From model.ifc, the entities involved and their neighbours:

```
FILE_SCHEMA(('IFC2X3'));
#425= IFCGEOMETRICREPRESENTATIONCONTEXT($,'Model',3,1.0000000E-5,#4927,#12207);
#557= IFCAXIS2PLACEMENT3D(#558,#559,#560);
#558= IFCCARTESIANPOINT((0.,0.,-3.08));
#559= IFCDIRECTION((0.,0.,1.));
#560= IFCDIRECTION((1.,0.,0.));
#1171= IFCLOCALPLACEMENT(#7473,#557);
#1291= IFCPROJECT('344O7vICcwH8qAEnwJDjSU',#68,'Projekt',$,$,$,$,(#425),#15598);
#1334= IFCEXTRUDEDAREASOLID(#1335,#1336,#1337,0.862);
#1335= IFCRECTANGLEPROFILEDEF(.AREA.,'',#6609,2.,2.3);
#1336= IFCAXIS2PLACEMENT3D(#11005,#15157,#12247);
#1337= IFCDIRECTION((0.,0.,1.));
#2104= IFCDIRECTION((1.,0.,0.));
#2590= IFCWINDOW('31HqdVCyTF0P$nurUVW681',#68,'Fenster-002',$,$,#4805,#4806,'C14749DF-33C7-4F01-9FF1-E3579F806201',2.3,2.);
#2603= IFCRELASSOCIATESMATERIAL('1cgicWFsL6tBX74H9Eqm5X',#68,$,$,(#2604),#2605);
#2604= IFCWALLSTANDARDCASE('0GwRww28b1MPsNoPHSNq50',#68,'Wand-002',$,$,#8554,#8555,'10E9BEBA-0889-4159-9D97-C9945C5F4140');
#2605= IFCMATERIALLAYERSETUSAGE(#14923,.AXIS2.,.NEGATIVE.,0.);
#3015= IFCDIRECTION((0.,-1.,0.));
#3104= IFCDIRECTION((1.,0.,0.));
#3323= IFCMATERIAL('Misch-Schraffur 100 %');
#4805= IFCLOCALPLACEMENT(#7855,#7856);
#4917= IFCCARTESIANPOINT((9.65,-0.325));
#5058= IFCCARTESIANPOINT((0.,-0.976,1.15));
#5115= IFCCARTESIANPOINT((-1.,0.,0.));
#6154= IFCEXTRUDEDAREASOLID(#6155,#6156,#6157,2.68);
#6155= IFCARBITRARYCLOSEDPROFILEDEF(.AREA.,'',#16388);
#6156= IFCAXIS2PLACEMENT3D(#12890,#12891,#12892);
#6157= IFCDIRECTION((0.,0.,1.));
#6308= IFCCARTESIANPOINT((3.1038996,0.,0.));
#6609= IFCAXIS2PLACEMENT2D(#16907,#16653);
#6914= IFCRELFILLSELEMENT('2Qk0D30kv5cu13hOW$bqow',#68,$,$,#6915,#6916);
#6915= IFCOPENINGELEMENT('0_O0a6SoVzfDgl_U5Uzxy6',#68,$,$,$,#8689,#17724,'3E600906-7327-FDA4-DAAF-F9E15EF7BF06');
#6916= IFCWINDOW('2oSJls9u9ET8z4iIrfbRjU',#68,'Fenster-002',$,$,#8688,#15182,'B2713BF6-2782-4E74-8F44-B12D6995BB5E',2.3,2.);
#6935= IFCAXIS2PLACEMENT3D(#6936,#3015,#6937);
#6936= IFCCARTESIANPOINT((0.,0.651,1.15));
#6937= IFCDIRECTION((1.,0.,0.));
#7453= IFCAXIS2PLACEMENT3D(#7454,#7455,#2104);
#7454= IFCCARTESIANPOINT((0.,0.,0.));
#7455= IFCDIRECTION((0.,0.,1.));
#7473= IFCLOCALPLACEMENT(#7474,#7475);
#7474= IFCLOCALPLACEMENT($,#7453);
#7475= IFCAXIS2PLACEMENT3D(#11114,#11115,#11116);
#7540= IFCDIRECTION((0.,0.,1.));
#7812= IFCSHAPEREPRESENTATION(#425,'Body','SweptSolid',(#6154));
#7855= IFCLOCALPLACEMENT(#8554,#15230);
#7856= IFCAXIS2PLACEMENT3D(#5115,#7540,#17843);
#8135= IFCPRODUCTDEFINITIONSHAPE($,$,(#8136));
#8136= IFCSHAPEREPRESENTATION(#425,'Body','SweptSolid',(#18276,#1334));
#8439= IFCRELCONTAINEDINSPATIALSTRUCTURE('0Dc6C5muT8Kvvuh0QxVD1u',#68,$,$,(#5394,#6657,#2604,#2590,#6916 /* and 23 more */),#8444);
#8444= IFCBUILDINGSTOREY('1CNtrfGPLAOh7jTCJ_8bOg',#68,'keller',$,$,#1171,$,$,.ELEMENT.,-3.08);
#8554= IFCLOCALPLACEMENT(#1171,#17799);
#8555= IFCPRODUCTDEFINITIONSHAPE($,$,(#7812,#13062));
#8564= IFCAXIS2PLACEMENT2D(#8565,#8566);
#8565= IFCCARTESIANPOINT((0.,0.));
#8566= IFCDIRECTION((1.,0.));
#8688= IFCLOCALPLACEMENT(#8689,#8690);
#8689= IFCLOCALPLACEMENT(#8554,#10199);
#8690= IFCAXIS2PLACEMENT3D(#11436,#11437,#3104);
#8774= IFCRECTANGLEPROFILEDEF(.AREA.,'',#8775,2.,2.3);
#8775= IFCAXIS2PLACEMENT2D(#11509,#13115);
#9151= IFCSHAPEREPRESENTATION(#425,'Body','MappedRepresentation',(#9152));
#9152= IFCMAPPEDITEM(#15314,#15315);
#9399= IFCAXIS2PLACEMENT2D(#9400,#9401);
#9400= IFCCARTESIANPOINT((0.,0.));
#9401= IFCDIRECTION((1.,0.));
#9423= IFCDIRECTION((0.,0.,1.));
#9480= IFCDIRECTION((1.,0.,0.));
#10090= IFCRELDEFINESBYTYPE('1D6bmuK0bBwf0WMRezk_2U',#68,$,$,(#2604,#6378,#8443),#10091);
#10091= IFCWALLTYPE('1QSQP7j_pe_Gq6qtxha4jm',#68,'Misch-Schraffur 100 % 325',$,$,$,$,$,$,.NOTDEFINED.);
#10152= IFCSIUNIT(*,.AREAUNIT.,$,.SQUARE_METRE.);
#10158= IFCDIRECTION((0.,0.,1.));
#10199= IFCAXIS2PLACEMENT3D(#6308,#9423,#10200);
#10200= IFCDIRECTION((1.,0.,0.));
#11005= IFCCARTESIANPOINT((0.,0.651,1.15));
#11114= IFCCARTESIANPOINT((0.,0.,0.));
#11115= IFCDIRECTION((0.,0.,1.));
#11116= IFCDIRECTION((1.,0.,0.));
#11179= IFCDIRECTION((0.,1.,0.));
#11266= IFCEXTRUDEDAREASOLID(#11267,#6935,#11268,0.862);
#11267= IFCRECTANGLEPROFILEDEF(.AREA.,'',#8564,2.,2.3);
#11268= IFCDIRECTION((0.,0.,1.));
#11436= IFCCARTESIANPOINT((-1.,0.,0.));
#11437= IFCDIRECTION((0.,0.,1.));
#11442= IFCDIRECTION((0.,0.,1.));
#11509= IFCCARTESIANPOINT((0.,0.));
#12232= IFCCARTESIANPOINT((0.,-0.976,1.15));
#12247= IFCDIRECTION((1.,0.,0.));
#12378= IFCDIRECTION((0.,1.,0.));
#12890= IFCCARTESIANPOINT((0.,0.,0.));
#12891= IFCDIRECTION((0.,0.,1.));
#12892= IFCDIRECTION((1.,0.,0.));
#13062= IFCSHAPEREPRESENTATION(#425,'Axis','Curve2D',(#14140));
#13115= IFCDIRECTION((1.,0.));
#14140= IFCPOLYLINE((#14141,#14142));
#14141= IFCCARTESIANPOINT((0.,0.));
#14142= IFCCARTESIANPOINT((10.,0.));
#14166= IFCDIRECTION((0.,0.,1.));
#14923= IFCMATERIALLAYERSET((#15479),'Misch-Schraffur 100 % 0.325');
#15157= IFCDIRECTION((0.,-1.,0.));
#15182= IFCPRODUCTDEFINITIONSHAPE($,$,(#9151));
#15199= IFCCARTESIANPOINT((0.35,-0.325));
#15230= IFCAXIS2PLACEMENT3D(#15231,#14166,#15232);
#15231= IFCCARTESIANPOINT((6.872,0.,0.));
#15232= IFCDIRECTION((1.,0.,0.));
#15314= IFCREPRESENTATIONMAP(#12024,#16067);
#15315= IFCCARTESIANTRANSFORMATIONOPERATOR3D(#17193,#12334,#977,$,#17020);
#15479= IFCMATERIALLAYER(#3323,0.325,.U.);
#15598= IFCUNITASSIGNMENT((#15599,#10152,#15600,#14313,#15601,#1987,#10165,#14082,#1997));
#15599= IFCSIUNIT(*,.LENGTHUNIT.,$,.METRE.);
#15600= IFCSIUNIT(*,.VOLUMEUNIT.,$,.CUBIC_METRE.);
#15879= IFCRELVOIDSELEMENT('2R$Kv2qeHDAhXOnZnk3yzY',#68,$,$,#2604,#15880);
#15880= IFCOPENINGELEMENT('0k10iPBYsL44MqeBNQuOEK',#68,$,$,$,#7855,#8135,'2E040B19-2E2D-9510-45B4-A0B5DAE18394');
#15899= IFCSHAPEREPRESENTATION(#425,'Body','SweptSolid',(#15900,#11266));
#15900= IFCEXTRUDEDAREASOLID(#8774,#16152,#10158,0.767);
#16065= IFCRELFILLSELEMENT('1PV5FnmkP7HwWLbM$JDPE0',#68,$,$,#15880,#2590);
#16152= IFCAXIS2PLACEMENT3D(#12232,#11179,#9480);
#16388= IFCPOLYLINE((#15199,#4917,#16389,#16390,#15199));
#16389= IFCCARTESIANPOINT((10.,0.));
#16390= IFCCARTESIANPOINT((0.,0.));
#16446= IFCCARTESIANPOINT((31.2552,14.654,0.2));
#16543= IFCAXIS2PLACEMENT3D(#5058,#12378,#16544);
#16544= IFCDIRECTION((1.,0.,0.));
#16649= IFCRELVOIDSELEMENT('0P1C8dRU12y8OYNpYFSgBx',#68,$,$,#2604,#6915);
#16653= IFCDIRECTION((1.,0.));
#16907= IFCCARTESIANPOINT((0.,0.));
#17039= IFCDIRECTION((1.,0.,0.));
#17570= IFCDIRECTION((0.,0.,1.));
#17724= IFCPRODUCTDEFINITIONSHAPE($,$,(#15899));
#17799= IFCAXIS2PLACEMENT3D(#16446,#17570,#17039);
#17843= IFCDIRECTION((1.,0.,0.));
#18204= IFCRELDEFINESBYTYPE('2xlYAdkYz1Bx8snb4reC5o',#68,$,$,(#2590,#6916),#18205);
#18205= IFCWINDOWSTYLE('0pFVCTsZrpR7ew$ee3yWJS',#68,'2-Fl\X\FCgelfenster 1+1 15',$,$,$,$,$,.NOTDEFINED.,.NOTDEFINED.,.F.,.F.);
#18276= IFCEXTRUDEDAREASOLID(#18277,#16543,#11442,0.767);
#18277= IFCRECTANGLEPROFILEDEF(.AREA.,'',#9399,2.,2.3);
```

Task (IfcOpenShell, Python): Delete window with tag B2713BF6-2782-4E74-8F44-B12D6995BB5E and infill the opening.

```python
import ifcopenshell
import ifcopenshell.api.feature
import ifcopenshell.api.root
import ifcopenshell.geom
import ifcopenshell.util.shape

model = ifcopenshell.open("model.ifc")
settings = ifcopenshell.geom.settings()


def volume(element):
    """Net volume in cubic metres, openings subtracted."""
    shape = ifcopenshell.geom.create_shape(settings, element)
    return ifcopenshell.util.shape.get_volume(shape.geometry)


window = model.by_guid("2oSJls9u9ET8z4iIrfbRjU")
opening = window.FillsVoids[0].RelatingOpeningElement
wall = opening.VoidsElements[0].RelatingBuildingElement
before = volume(wall)

ifcopenshell.api.root.remove_product(model, product=window)
ifcopenshell.api.feature.remove_feature(model, feature=opening)

after = volume(wall)

print(f"wall volume {before:.3f} -> {after:.3f} m3")

model.write("model_updated.ifc")
```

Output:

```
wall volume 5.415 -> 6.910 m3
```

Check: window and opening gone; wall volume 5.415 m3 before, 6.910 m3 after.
